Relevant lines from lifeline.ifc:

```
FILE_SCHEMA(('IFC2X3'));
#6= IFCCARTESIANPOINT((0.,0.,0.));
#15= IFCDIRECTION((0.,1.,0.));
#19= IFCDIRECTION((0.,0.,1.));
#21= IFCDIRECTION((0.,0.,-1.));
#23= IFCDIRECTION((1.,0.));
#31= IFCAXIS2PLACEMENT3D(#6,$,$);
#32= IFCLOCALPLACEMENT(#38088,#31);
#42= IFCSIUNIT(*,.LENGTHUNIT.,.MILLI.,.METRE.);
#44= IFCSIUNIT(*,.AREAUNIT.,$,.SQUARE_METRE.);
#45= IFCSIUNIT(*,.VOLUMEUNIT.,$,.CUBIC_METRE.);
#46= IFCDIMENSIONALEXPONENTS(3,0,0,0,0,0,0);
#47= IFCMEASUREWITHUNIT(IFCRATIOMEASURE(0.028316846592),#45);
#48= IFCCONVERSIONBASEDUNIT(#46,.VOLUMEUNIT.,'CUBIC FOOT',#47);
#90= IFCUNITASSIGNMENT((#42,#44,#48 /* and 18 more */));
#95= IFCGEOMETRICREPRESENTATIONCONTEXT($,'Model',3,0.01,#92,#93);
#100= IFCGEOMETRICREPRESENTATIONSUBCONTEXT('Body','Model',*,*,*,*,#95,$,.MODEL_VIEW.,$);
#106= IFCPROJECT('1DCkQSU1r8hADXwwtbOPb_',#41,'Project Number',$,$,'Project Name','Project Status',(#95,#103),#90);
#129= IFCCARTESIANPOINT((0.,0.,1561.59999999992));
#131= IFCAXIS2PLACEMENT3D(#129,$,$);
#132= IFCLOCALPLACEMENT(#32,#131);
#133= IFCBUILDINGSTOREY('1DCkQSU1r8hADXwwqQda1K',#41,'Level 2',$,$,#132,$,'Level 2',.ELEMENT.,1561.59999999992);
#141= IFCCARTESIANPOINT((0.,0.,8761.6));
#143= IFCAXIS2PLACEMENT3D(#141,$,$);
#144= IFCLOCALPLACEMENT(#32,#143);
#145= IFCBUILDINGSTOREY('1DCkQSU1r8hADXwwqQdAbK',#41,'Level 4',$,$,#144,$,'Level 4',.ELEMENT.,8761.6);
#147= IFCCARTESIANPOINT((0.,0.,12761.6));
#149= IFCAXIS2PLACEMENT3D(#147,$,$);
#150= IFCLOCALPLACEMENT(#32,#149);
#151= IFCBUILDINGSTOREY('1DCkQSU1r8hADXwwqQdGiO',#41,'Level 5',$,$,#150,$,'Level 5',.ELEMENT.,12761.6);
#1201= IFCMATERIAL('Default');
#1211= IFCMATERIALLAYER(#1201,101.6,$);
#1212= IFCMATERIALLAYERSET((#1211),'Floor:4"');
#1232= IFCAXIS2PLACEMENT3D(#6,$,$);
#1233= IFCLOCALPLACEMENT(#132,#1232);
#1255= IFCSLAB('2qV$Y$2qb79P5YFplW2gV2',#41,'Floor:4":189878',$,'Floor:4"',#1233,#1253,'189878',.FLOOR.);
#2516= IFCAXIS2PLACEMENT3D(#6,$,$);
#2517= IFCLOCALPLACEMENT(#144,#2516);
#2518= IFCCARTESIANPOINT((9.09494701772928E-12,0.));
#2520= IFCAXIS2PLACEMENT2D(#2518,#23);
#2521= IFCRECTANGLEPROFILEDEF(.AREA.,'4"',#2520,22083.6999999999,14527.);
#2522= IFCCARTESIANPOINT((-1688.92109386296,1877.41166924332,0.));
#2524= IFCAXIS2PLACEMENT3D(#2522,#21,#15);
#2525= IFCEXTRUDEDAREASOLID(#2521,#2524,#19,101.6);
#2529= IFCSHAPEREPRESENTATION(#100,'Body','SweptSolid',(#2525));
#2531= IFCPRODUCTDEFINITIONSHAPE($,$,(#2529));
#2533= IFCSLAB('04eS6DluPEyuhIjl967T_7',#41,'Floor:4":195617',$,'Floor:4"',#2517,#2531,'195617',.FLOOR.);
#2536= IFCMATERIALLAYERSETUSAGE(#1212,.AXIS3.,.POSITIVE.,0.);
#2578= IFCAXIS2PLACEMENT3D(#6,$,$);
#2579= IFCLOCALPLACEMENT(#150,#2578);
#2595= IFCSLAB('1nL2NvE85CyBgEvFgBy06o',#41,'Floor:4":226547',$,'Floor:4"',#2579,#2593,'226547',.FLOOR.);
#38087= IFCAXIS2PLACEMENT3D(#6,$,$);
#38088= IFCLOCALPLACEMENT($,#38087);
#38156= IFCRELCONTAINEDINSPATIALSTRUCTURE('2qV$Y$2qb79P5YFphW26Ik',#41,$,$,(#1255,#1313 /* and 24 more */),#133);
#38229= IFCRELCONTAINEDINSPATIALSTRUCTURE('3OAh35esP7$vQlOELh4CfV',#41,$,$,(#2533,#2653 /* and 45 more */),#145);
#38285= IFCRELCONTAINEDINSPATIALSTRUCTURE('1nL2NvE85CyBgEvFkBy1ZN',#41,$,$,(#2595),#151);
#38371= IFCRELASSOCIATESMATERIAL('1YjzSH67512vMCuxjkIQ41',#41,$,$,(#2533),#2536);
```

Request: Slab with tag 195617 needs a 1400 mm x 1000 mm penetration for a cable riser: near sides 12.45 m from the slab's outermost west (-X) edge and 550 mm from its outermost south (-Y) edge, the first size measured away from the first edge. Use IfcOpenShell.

```python
import numpy as np
import ifcopenshell
import ifcopenshell.api.feature
import ifcopenshell.api.geometry
import ifcopenshell.api.root
import ifcopenshell.geom
import ifcopenshell.util.placement
import ifcopenshell.util.representation
import ifcopenshell.util.shape
import ifcopenshell.util.unit

model = ifcopenshell.open("lifeline.ifc")
unit_scale = ifcopenshell.util.unit.calculate_unit_scale(model)
settings = ifcopenshell.geom.settings()


def volume(element):
    """Net volume in cubic metres, openings subtracted."""
    shape = ifcopenshell.geom.create_shape(settings, element)
    return ifcopenshell.util.shape.get_volume(shape.geometry)


slab = model.by_id(2533)
before = volume(slab)

# Extent in the slab's own axes, in metres. The edges named are its -X and -Y sides.
slab_shape = ifcopenshell.geom.create_shape(settings, slab)
vertices = ifcopenshell.util.shape.get_vertices(slab_shape.geometry)
x_min, y_min, bottom = vertices.min(axis=0)
top = vertices[:, 2].max()

opening = ifcopenshell.api.root.create_entity(model, ifc_class="IfcOpeningElement", name="Cable riser opening")
context = ifcopenshell.util.representation.get_context(model, "Model", "Body", "MODEL_VIEW")
width, depth = 1.4, 1
outline = [(0.0, 0.0), (width, 0.0), (width, depth), (0.0, depth), (0.0, 0.0)]
# Overshoot both faces by 50 mm so the cut is clean.
shape = ifcopenshell.api.geometry.add_slab_representation(
    model, context=context, depth=top - bottom + 0.1, polyline=outline
)
ifcopenshell.api.geometry.assign_representation(model, product=opening, representation=shape)

matrix = ifcopenshell.util.placement.get_local_placement(slab.ObjectPlacement)
matrix[:, 3] = matrix @ np.append(np.array([x_min + 12.45, y_min + 0.55, bottom - 0.05]) / unit_scale, 1.0)
ifcopenshell.api.geometry.edit_object_placement(model, product=opening, matrix=matrix, is_si=False)
ifcopenshell.api.feature.add_feature(model, feature=opening, element=slab)

after = volume(slab)

print(f"slab volume {before:.3f} -> {after:.3f} m3")

model.write("lifeline_rev.ifc")
```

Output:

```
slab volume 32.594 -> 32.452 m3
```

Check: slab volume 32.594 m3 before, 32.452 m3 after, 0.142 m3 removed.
